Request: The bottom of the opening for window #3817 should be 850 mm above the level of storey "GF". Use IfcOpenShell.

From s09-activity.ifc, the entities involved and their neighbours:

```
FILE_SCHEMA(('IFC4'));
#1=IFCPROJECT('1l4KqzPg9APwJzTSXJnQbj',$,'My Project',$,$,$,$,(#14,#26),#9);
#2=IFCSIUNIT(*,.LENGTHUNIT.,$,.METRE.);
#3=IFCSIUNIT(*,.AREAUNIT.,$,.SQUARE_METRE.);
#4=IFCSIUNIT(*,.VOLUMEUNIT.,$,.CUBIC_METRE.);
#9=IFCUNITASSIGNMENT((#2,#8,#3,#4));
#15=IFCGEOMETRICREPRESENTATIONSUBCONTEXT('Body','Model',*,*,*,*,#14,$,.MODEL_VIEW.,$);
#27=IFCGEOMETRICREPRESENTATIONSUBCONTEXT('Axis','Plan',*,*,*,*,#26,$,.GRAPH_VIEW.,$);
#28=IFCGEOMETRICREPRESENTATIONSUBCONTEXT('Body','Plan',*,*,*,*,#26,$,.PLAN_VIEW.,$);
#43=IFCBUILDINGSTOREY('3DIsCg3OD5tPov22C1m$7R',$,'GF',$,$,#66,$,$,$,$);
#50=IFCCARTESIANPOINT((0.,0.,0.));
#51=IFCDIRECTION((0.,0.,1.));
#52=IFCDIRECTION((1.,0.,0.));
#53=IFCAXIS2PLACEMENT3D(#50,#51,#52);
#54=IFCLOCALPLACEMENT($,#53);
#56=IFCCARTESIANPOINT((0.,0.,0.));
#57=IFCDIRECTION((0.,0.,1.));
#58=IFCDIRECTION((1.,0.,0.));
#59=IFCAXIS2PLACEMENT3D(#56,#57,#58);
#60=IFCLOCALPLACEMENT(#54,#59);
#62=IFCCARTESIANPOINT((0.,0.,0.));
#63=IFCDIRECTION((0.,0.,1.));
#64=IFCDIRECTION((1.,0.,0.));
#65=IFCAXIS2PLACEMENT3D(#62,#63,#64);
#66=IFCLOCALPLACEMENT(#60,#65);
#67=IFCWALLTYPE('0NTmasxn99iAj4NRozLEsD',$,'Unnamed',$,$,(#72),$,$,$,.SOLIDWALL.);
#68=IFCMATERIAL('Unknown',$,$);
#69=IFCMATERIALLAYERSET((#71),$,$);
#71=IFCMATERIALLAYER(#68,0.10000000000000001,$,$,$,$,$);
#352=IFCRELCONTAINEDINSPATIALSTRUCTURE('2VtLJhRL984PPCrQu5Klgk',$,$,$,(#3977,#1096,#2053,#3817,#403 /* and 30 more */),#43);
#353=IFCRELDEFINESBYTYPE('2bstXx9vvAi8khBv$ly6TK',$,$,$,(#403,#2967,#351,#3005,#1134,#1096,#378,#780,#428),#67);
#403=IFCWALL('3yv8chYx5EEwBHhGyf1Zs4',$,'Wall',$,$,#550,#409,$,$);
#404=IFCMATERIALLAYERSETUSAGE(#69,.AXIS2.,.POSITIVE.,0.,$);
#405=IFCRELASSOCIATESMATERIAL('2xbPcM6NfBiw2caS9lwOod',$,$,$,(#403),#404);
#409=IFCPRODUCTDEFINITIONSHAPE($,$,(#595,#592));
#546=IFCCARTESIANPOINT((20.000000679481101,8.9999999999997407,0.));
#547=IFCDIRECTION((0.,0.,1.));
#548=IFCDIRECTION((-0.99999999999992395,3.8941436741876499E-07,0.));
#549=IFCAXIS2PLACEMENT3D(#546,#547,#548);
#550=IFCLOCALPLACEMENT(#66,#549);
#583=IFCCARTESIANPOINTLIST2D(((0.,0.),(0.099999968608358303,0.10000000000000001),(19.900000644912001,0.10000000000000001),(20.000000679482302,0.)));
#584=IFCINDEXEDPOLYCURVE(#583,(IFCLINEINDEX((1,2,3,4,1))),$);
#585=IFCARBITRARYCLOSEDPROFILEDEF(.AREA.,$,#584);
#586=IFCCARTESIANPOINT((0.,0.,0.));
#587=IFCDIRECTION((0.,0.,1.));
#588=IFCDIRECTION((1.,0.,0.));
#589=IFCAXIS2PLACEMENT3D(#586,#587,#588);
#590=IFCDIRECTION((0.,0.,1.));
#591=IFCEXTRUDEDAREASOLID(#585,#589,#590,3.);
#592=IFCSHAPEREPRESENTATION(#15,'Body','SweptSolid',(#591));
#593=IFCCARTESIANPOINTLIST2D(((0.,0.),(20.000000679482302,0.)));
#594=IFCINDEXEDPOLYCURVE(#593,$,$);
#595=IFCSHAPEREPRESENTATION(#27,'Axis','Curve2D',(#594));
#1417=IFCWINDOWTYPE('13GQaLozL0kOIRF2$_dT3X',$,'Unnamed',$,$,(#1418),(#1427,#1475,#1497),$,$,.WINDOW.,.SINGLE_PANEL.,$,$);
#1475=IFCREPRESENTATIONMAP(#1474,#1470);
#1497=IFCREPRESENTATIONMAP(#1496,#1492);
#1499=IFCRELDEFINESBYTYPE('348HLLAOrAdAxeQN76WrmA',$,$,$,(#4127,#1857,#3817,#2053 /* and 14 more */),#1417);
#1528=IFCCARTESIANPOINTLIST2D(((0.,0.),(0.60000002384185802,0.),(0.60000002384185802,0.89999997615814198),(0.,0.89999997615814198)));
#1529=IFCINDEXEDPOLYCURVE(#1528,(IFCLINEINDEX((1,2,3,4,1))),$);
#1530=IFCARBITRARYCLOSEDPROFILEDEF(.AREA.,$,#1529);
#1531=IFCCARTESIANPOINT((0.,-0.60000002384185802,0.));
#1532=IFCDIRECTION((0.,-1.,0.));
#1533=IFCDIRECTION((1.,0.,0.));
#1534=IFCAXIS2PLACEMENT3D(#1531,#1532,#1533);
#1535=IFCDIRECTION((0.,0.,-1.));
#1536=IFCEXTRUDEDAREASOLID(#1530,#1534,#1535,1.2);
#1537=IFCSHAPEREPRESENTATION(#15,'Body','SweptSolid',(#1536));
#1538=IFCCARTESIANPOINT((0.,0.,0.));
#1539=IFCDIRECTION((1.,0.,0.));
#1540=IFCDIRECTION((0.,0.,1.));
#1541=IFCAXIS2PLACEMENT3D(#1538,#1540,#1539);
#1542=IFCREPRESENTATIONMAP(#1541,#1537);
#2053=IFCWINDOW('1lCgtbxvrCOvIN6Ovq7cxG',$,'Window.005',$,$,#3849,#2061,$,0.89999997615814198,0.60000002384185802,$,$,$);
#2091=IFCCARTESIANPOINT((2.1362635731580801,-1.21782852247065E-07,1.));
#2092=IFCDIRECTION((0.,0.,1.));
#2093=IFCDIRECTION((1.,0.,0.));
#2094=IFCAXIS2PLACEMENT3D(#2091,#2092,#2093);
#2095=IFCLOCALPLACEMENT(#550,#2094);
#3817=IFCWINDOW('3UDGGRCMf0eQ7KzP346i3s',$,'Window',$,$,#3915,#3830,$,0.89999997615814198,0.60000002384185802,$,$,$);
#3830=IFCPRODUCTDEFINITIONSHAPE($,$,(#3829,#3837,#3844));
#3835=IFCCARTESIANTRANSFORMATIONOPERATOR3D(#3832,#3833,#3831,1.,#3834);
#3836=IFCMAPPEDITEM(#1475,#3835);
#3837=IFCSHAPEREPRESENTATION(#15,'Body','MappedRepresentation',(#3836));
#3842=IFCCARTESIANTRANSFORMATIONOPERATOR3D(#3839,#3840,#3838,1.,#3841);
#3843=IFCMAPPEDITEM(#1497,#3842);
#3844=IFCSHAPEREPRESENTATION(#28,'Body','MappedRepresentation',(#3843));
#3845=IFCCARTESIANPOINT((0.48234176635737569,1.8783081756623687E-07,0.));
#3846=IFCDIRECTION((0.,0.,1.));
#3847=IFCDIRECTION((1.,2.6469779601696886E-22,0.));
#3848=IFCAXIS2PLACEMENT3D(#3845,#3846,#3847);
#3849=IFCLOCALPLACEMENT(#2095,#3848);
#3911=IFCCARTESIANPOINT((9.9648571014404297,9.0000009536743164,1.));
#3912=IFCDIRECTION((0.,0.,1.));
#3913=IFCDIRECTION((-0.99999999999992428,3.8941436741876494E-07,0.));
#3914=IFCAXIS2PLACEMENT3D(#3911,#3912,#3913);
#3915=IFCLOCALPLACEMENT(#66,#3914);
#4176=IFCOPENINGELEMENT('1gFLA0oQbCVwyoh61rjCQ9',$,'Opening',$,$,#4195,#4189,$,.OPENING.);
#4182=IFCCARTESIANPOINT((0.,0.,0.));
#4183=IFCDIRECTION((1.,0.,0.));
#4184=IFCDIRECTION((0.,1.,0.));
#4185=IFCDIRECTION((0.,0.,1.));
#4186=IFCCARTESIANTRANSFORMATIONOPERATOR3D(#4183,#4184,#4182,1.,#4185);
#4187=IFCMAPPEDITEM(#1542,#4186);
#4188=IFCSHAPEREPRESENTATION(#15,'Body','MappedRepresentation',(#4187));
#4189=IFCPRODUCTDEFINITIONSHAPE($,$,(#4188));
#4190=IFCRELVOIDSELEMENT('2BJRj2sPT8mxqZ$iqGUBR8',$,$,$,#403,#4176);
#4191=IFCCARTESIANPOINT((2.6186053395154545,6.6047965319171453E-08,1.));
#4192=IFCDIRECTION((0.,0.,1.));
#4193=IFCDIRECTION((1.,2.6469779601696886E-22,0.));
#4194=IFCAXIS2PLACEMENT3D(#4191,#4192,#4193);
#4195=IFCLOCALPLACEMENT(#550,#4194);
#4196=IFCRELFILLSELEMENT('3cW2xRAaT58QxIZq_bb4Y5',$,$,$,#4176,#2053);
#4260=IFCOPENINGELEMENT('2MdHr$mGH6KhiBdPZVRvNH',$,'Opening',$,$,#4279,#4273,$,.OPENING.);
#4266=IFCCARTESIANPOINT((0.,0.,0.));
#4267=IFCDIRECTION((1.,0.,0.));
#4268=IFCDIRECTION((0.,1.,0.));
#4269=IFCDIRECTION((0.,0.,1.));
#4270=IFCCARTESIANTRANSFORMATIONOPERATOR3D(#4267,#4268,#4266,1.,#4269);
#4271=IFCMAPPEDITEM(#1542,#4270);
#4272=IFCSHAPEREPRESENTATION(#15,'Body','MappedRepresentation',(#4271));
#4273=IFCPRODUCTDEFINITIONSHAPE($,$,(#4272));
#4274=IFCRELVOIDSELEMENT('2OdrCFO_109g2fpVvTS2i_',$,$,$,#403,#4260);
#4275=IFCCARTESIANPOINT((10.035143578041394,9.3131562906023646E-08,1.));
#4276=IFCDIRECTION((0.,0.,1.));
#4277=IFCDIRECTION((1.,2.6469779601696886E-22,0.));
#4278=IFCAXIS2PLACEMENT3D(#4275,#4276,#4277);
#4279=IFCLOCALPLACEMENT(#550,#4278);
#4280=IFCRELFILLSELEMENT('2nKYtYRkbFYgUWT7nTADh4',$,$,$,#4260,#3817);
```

```python
import numpy as np
import ifcopenshell
import ifcopenshell.api.geometry
import ifcopenshell.geom
import ifcopenshell.util.element
import ifcopenshell.util.placement
import ifcopenshell.util.shape
import ifcopenshell.util.unit

model = ifcopenshell.open("s09-activity.ifc")
unit_scale = ifcopenshell.util.unit.calculate_unit_scale(model)

window = model.by_id(3817)
opening = window.FillsVoids[0].RelatingOpeningElement
storey = ifcopenshell.util.element.get_container(window, ifc_class="IfcBuildingStorey")
level = ifcopenshell.util.placement.get_local_placement(storey.ObjectPlacement)[2, 3]

# The opening's origin need not be at the sill, so measure its lowest point.
shape = ifcopenshell.geom.create_shape(ifcopenshell.geom.settings(), opening)
bottom = ifcopenshell.util.shape.get_shape_bottom_elevation(shape, shape.geometry) / unit_scale
dz = level + 0.85 / unit_scale - bottom

shift = np.array([0.0, 0.0, dz])
# The window is not placed relative to its opening, so move both.
for product in (opening, window):
    matrix = ifcopenshell.util.placement.get_local_placement(product.ObjectPlacement)
    matrix[:3, 3] += shift
    ifcopenshell.api.geometry.edit_object_placement(model, product=product, matrix=matrix, is_si=False)

print(f"moved by {dz * unit_scale:+.3f} m")

model.write("s09-activity_edited.ifc")
```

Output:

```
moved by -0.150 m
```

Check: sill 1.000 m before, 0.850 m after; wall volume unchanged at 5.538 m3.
